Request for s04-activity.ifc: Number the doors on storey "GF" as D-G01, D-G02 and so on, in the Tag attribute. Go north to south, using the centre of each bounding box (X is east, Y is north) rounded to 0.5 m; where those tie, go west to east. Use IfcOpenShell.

First a look at what the model holds.

```python
import ifcopenshell
import ifcopenshell.util.element
import ifcopenshell.util.placement

model = ifcopenshell.open("s04-activity.ifc")
print(model.schema)
storey = next(s for s in model.by_type("IfcBuildingStorey") if s.Name == "GF")
doors = [e for e in ifcopenshell.util.element.get_decomposition(storey) if e.is_a("IfcDoor")]
for e in sorted(doors, key=lambda e: e.id()):
    origin = ifcopenshell.util.placement.get_local_placement(e.ObjectPlacement)[:3, 3]
    print(e.id(), e.Tag, e.Name, origin.round(2) + 0.0, sep=" | ")
```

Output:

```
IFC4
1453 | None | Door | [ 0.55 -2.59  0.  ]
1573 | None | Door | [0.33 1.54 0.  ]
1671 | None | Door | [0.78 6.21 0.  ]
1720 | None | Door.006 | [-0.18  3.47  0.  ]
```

```python
import ifcopenshell
import ifcopenshell.geom
import ifcopenshell.util.element
import ifcopenshell.util.shape

model = ifcopenshell.open("s04-activity.ifc")
settings = ifcopenshell.geom.settings()
settings.set("use-world-coords", True)


def centre(element):
    shape = ifcopenshell.geom.create_shape(settings, element)
    return ifcopenshell.util.shape.get_bbox_centroid(shape.geometry)


storey = next(s for s in model.by_type("IfcBuildingStorey") if s.Name == "GF")
doors = [e for e in ifcopenshell.util.element.get_decomposition(storey) if e.is_a("IfcDoor")]

# Insertion points can sit at a corner or the storey origin, so sort by the geometry (in metres).
centres = {e: centre(e) for e in doors}
doors.sort(key=lambda e: (-round(centres[e][1] / 0.5), centres[e][0]))

for i, e in enumerate(doors, start=1):
    number = f"D-G{i:02d}"
    e.Tag = number
    print(e.id(), number)

model.write("s04-activity_v2.ifc")
```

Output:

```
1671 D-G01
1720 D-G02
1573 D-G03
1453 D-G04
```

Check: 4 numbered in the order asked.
